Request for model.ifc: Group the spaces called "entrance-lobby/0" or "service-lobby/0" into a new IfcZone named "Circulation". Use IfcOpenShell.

First a look at what the model holds.

```python
import ifcopenshell

model = ifcopenshell.open("model.ifc")
print(model.schema)
seen = {}
for space in model.by_type("IfcSpace"):
    seen[space.Name] = seen.get(space.Name, 0) + 1
for name, count in sorted(seen.items(), key=str):
    print(count, "x", name)
print("zones:", [z.Name for z in model.by_type("IfcZone")][:20])
```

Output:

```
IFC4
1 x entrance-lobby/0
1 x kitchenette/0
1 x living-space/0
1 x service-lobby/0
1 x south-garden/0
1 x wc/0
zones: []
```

```python
import ifcopenshell
import ifcopenshell.api.group
import ifcopenshell.api.root

model = ifcopenshell.open("model.ifc")

names = {"entrance-lobby/0", "service-lobby/0"}
spaces = [s for s in model.by_type("IfcSpace") if s.Name in names]

zone = ifcopenshell.api.root.create_entity(model, ifc_class="IfcZone", name="Circulation")
ifcopenshell.api.group.assign_group(model, products=spaces, group=zone)
print(len(spaces), "spaces in", zone.Name)

model.write("model_updated.ifc")
```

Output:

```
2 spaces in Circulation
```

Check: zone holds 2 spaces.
